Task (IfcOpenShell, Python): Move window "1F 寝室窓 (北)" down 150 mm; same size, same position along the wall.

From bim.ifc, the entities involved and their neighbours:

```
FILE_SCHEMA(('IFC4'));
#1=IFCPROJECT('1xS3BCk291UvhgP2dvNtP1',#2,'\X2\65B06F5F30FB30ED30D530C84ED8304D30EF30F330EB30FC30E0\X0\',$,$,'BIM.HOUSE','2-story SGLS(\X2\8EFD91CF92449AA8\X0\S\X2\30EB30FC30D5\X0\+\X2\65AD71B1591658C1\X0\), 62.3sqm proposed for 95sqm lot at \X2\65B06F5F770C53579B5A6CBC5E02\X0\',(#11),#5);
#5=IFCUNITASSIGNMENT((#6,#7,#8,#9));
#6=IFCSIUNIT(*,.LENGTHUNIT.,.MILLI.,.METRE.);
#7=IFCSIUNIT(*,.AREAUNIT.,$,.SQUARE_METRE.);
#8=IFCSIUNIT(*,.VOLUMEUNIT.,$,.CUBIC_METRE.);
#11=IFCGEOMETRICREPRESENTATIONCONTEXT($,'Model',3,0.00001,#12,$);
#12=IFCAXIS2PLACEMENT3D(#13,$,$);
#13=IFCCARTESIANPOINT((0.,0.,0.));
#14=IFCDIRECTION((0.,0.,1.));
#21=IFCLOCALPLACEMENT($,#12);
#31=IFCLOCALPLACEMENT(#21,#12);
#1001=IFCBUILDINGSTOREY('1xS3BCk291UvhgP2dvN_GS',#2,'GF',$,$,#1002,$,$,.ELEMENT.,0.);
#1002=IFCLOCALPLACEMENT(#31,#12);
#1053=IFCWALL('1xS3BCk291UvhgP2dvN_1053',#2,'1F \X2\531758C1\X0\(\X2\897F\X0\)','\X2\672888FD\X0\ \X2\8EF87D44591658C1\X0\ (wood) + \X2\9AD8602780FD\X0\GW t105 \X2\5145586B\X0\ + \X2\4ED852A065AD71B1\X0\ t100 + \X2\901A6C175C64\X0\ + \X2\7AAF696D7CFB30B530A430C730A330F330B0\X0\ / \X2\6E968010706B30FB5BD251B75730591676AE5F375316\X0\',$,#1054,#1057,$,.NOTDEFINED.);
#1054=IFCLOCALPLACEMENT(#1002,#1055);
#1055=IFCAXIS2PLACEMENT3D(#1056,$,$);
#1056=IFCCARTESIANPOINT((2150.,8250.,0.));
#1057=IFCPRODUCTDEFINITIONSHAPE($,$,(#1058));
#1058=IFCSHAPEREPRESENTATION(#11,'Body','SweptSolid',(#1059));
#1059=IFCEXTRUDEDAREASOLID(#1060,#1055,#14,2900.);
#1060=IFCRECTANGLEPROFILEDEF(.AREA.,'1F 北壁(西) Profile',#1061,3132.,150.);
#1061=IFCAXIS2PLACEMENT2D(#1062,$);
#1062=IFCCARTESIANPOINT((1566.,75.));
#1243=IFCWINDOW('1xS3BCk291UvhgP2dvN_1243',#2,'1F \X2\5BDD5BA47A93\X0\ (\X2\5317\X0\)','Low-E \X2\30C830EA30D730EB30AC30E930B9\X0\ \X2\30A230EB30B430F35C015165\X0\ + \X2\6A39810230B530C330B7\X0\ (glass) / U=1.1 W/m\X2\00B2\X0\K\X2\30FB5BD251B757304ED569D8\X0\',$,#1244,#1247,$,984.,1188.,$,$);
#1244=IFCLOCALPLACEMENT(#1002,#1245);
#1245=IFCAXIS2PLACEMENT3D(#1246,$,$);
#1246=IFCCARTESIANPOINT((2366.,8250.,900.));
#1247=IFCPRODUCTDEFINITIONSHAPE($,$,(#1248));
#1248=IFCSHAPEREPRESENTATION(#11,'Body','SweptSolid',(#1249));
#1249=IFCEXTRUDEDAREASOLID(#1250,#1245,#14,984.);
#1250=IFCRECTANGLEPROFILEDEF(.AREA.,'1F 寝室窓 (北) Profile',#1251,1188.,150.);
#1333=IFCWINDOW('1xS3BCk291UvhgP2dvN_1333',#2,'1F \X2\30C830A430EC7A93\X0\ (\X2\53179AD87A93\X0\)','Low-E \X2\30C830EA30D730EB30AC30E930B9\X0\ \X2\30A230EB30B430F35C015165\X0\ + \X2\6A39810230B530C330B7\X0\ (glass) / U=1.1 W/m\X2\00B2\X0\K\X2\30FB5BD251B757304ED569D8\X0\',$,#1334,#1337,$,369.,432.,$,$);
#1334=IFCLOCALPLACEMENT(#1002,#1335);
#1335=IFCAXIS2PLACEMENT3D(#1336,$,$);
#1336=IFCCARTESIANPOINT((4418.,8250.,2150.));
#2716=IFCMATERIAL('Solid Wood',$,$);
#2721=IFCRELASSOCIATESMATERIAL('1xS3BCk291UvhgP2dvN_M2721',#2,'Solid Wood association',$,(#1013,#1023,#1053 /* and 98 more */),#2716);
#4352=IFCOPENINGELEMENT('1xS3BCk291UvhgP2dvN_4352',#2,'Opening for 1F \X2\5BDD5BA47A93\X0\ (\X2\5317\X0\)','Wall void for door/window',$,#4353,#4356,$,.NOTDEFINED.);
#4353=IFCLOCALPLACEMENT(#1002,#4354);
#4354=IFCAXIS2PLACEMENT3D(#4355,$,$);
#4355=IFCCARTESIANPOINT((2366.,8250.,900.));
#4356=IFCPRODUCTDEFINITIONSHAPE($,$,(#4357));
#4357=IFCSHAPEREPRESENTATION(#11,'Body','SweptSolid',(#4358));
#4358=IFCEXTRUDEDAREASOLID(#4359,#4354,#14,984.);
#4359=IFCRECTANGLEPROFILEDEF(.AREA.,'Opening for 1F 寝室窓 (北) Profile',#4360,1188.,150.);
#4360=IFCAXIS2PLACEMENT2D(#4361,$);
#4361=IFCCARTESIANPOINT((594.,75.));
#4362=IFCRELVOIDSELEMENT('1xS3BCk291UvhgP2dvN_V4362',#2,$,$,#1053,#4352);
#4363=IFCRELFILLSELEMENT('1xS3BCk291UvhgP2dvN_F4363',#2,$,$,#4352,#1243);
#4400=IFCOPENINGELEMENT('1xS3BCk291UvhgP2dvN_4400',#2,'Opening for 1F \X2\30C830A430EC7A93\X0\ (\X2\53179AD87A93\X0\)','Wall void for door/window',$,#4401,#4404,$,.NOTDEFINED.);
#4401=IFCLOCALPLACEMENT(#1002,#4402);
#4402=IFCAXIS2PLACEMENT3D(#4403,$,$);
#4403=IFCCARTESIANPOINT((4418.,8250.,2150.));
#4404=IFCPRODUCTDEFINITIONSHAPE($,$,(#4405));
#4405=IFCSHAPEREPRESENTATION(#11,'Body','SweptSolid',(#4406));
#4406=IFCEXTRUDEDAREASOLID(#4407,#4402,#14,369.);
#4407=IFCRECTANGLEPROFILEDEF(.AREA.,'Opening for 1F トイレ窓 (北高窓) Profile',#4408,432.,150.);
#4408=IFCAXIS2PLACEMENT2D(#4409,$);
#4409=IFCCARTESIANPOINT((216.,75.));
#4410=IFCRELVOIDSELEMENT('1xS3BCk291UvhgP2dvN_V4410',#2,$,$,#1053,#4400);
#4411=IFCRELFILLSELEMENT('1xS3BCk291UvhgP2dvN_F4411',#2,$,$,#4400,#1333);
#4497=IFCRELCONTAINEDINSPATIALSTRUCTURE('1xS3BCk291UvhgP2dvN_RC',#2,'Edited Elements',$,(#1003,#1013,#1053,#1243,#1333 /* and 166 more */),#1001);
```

```python
import numpy as np
import ifcopenshell
import ifcopenshell.api.geometry
import ifcopenshell.util.placement
import ifcopenshell.util.unit

model = ifcopenshell.open("bim.ifc")
unit_scale = ifcopenshell.util.unit.calculate_unit_scale(model)

window = model.by_guid("1xS3BCk291UvhgP2dvN_1243")
opening = window.FillsVoids[0].RelatingOpeningElement
dz = -0.15 / unit_scale

shift = np.array([0.0, 0.0, dz])
# The window is not placed relative to its opening, so move both.
for product in (opening, window):
    matrix = ifcopenshell.util.placement.get_local_placement(product.ObjectPlacement)
    matrix[:3, 3] += shift
    ifcopenshell.api.geometry.edit_object_placement(model, product=product, matrix=matrix, is_si=False)

print(f"moved by {dz * unit_scale:+.3f} m")

model.write("bim_edited.ifc")
```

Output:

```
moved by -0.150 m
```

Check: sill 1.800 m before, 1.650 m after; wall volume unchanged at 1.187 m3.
